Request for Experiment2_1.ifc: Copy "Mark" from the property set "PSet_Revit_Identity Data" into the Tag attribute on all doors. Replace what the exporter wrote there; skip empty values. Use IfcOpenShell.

First a look at what the model holds.

```python
import ifcopenshell
import ifcopenshell.util.element

model = ifcopenshell.open("Experiment2_1.ifc")
print(model.schema)
doors = model.by_type("IfcDoor")
print(len(doors), "doors")
for e in doors[:8]:
    source = ifcopenshell.util.element.get_pset(e, "PSet_Revit_Identity Data", "Mark")
    target = e.Tag
    print(e.id(), repr(source), repr(target), sep=" | ")
```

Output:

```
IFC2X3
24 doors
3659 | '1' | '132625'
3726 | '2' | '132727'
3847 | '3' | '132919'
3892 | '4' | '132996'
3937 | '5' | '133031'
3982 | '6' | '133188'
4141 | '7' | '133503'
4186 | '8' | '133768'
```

```python
import ifcopenshell
import ifcopenshell.util.element

model = ifcopenshell.open("Experiment2_1.ifc")

count = 0
for e in model.by_type("IfcDoor"):
    value = ifcopenshell.util.element.get_pset(e, "PSet_Revit_Identity Data", "Mark")
    current = e.Tag
    if not value or not value.strip() or current == value:
        continue
    e.Tag = value
    count += 1

print(count, "doors updated")

model.write("Experiment2_1_updated.ifc")
```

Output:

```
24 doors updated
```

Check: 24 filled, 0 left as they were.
